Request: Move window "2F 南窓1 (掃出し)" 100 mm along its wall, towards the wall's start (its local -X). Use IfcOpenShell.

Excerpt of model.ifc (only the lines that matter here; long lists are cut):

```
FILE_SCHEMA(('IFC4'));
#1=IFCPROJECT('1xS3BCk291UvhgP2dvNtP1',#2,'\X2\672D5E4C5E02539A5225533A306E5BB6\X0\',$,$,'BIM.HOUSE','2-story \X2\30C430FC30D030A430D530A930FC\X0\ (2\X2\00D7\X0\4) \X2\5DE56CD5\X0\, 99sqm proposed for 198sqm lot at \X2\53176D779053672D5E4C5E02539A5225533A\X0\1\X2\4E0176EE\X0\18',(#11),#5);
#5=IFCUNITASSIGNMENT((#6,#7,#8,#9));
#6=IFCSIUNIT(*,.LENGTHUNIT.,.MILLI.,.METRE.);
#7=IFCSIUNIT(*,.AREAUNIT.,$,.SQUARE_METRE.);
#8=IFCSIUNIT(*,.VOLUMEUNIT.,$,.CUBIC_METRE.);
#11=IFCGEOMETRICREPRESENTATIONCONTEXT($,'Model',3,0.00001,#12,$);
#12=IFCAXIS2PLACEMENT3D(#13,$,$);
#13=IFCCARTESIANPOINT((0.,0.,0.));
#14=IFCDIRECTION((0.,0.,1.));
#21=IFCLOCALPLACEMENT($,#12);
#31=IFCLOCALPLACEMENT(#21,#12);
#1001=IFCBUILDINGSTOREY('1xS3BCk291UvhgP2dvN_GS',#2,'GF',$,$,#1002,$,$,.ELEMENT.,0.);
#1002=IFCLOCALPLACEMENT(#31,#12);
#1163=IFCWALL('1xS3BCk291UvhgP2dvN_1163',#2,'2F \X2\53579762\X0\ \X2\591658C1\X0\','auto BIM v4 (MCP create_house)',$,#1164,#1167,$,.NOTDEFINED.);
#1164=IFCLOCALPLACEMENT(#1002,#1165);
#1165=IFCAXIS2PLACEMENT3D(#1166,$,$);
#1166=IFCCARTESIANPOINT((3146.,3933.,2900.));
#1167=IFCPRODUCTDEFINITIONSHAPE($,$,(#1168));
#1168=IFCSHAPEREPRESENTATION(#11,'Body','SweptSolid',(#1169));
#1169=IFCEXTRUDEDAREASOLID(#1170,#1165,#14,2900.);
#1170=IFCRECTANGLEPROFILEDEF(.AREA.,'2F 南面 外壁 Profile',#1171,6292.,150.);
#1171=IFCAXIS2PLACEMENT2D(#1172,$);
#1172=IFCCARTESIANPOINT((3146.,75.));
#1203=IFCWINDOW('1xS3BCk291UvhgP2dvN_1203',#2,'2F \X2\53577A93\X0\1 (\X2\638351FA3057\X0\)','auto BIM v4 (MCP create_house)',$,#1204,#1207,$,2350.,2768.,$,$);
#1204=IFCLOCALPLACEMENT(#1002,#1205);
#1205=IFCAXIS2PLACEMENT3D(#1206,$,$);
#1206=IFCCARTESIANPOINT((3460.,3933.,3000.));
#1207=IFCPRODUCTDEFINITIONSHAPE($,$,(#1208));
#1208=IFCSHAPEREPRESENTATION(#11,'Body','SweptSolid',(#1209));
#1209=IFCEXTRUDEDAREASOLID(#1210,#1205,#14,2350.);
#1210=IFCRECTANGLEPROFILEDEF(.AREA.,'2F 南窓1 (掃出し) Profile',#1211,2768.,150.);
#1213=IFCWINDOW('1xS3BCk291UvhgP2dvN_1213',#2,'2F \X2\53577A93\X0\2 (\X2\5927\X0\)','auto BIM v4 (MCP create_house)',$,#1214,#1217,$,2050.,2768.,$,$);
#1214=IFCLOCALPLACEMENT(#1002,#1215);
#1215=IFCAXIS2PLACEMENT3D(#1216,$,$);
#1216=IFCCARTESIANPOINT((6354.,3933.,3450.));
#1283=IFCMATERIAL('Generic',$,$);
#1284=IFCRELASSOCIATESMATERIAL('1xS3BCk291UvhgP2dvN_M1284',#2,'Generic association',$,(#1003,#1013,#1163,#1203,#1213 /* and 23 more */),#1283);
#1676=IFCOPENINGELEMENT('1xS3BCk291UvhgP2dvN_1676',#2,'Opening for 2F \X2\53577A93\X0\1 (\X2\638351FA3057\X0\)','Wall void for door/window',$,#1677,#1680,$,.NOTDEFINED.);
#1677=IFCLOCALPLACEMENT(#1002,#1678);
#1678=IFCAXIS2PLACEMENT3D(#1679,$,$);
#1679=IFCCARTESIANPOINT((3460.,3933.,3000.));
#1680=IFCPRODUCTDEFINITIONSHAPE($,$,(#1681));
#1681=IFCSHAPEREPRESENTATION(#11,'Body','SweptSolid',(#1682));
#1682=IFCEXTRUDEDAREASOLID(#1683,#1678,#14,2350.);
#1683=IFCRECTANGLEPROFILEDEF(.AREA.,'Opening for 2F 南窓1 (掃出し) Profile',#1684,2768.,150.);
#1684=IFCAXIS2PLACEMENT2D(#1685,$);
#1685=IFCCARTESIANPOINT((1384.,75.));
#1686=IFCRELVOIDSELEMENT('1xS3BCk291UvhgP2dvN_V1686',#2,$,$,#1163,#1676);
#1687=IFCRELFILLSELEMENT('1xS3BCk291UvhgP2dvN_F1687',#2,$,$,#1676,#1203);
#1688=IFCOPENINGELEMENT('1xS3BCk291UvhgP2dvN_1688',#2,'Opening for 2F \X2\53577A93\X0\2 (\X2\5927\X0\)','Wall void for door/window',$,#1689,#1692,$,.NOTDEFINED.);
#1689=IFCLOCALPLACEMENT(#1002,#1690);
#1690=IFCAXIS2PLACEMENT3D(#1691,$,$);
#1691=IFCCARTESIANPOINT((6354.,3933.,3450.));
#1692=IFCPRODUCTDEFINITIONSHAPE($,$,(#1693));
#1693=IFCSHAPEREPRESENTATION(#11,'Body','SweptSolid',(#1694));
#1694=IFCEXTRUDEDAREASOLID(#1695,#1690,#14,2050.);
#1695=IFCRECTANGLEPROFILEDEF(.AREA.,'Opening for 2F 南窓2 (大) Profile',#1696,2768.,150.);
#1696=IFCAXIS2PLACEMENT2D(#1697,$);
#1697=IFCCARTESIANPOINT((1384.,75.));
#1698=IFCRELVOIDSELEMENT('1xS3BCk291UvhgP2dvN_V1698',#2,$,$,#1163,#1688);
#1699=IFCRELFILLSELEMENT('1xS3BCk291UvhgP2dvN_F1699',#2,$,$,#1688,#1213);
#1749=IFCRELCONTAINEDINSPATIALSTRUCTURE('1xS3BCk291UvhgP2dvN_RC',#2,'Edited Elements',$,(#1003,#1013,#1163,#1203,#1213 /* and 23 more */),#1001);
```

```python
import ifcopenshell
import ifcopenshell.api.geometry
import ifcopenshell.util.placement
import ifcopenshell.util.unit

model = ifcopenshell.open("model.ifc")
unit_scale = ifcopenshell.util.unit.calculate_unit_scale(model)

window = model.by_guid("1xS3BCk291UvhgP2dvN_1203")
opening = window.FillsVoids[0].RelatingOpeningElement
wall = opening.VoidsElements[0].RelatingBuildingElement

wall_matrix = ifcopenshell.util.placement.get_local_placement(wall.ObjectPlacement)
shift = wall_matrix[:3, 0] * -0.1 / unit_scale
before = ifcopenshell.util.placement.get_local_placement(window.ObjectPlacement)[:3, 3].copy()

# The window is not placed relative to its opening, so move both.
for product in (opening, window):
    matrix = ifcopenshell.util.placement.get_local_placement(product.ObjectPlacement)
    matrix[:3, 3] += shift
    ifcopenshell.api.geometry.edit_object_placement(model, product=product, matrix=matrix, is_si=False)

after = ifcopenshell.util.placement.get_local_placement(window.ObjectPlacement)[:3, 3]
print("window moved by", (after - before).round(3) + 0.0)

model.write("model_v2.ifc")
```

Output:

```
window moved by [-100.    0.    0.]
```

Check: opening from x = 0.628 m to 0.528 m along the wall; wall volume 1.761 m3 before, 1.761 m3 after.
